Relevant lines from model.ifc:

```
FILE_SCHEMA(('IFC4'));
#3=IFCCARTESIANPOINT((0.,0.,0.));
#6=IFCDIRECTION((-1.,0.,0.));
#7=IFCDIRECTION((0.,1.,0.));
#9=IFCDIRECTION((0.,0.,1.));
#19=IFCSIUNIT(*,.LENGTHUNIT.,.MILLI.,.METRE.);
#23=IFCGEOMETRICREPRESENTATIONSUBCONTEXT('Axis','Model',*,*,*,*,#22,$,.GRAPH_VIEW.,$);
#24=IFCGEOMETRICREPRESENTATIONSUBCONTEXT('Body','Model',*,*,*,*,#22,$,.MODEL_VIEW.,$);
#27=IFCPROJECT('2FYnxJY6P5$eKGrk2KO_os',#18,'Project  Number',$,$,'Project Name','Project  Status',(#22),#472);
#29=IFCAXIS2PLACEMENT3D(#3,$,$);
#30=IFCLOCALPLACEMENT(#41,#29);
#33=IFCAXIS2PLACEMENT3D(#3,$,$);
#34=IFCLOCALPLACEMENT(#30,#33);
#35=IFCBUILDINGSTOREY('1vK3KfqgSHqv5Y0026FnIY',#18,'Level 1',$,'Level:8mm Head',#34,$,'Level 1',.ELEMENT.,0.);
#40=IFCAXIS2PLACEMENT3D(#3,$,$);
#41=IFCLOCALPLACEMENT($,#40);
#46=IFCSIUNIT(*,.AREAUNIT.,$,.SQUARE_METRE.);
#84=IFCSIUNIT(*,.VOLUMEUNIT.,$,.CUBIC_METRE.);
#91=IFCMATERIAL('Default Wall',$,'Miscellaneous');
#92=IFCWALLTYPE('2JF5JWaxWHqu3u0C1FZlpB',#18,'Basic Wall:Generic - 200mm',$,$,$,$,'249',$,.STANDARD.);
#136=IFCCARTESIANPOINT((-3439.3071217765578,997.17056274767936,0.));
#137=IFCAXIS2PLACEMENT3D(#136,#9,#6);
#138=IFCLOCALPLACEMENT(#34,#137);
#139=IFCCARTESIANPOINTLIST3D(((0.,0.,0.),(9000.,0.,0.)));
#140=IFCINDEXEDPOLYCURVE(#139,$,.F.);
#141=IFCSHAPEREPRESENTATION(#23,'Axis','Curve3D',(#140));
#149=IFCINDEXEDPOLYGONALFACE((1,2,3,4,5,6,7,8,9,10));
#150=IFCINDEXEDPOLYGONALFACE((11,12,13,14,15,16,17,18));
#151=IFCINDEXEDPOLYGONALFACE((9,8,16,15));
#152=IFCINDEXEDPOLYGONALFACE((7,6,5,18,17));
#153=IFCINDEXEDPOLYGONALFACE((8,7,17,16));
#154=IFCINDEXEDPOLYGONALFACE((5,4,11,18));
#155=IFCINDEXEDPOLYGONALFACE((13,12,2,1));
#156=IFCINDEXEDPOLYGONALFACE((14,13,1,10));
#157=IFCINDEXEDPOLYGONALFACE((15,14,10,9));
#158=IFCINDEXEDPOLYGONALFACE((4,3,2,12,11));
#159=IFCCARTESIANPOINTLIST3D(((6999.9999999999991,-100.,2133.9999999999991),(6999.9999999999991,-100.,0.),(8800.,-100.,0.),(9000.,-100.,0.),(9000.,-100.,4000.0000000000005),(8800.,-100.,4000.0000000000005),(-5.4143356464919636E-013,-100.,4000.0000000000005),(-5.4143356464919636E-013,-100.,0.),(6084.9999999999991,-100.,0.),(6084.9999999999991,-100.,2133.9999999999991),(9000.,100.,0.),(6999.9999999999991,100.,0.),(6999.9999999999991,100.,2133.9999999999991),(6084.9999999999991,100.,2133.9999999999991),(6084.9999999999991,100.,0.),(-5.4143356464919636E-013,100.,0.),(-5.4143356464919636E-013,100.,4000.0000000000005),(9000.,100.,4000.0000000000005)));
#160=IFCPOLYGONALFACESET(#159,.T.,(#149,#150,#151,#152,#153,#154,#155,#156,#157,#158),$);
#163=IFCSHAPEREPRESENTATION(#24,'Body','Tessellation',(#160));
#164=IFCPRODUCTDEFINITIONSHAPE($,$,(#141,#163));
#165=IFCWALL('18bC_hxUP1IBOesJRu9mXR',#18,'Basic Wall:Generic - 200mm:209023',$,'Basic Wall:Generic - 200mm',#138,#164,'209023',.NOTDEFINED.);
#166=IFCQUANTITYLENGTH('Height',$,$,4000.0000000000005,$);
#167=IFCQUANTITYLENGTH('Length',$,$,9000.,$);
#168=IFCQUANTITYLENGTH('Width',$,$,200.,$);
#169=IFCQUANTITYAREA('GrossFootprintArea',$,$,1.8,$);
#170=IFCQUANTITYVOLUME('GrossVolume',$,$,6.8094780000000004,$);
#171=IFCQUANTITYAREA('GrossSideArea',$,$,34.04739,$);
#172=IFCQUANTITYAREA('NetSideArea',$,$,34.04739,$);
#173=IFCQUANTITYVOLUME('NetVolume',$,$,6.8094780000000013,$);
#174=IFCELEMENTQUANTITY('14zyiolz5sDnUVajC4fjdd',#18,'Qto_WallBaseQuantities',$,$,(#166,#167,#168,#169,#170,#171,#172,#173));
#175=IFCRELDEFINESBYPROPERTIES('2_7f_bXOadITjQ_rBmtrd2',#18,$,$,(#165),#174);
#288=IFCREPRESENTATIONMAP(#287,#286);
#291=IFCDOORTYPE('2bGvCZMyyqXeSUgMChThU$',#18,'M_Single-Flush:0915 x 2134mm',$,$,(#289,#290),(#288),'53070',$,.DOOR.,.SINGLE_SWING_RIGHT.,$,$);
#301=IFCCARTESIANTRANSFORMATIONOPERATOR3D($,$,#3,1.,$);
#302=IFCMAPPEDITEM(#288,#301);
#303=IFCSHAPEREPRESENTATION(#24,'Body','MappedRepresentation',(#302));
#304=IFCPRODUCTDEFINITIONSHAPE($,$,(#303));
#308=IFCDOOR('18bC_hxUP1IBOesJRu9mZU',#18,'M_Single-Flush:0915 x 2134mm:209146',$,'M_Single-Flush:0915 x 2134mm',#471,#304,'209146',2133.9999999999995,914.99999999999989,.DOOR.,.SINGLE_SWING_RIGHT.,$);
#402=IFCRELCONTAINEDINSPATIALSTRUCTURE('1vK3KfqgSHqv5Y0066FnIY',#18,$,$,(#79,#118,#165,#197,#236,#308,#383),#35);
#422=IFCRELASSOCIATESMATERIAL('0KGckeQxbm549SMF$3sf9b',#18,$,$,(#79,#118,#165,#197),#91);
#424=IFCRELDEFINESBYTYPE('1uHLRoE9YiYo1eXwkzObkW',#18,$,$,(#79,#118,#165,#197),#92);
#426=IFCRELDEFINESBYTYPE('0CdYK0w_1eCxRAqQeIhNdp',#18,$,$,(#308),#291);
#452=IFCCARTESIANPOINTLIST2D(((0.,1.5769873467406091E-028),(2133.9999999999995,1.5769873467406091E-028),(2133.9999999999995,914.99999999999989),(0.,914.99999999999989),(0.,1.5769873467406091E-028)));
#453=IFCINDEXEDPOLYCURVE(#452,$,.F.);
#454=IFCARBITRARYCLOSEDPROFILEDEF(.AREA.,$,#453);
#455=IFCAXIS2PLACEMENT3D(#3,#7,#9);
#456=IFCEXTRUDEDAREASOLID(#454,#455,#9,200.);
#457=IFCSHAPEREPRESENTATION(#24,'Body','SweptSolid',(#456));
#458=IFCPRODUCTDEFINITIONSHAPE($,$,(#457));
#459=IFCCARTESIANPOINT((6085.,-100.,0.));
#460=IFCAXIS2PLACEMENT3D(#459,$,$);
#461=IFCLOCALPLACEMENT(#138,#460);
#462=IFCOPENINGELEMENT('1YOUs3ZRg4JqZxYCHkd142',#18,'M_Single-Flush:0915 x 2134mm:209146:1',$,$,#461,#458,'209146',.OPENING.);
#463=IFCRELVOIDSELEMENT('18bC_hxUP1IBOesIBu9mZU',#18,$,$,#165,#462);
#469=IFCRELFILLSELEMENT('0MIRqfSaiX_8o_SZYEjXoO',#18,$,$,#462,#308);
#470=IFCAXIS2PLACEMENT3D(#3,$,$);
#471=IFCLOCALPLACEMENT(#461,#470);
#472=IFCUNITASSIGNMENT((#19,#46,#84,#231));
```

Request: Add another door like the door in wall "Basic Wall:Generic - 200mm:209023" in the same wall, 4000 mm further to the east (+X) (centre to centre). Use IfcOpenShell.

```python
import ifcopenshell
import ifcopenshell.api.feature
import ifcopenshell.api.geometry
import ifcopenshell.api.pset
import ifcopenshell.api.root
import ifcopenshell.geom
import ifcopenshell.util.element
import ifcopenshell.util.placement
import ifcopenshell.util.shape
import ifcopenshell.util.unit

model = ifcopenshell.open("model.ifc")
unit_scale = ifcopenshell.util.unit.calculate_unit_scale(model)
area_scale = ifcopenshell.util.unit.calculate_unit_scale(model, "AREAUNIT")
volume_scale = ifcopenshell.util.unit.calculate_unit_scale(model, "VOLUMEUNIT")
settings = ifcopenshell.geom.settings()


def volume(element):
    """Net volume in cubic metres, openings subtracted."""
    shape = ifcopenshell.geom.create_shape(settings, element)
    return ifcopenshell.util.shape.get_volume(shape.geometry)


def reuse_history(source, copy):
    """copy_class also copies each property set's owner history, people and application; keep the originals."""
    for rel in copy.IsDefinedBy:
        if rel.is_a("IfcRelDefinesByProperties") and (history := rel.RelatingPropertyDefinition.OwnerHistory):
            rel.RelatingPropertyDefinition.OwnerHistory = source.OwnerHistory
            ifcopenshell.util.element.remove_deep2(model, history)


door = model.by_guid("18bC_hxUP1IBOesJRu9mZU")
opening = door.FillsVoids[0].RelatingOpeningElement
wall = opening.VoidsElements[0].RelatingBuildingElement
before = volume(wall)
shift = ifcopenshell.util.placement.get_local_placement(wall.ObjectPlacement)[:3, 0] * -4 / unit_scale

# copy_class copies the void relationship, type, container and properties, but no geometry.
new_opening = ifcopenshell.api.root.copy_class(model, product=opening)
new_opening.Representation = ifcopenshell.util.element.copy_deep(
    model, opening.Representation, exclude=["IfcGeometricRepresentationContext", "IfcRepresentationMap"]
)
new_opening.Name = "M_Single-Flush:0915 x 2134mm"
new_opening.Tag = None
reuse_history(opening, new_opening)
new_door = ifcopenshell.api.root.copy_class(model, product=door)
new_door.Representation = ifcopenshell.util.element.copy_deep(
    model, door.Representation, exclude=["IfcGeometricRepresentationContext", "IfcRepresentationMap"]
)
new_door.Name = "M_Single-Flush:0915 x 2134mm"
new_door.Tag = None
reuse_history(door, new_door)
ifcopenshell.api.feature.add_filling(model, opening=new_opening, element=new_door)

for old, new in ((opening, new_opening), (door, new_door)):
    matrix = ifcopenshell.util.placement.get_local_placement(old.ObjectPlacement)
    matrix[:3, 3] += shift
    ifcopenshell.api.geometry.edit_object_placement(model, product=new, matrix=matrix, is_si=False)

after = volume(wall)
thickness = 0.2  # wall thickness in metres

# Update the wall's stored quantities.
qto = model.by_id(ifcopenshell.util.element.get_pset(wall, "Qto_WallBaseQuantities", should_inherit=False)["id"])
ifcopenshell.api.pset.edit_qto(model, qto=qto, properties={
    "NetSideArea": after / thickness / area_scale,
    "NetVolume": after / volume_scale,
})

print(f"wall volume {before:.3f} -> {after:.3f} m3")

model.write("model_edited.ifc")
```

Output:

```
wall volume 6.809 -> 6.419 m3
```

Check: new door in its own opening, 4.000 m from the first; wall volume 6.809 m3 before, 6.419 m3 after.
